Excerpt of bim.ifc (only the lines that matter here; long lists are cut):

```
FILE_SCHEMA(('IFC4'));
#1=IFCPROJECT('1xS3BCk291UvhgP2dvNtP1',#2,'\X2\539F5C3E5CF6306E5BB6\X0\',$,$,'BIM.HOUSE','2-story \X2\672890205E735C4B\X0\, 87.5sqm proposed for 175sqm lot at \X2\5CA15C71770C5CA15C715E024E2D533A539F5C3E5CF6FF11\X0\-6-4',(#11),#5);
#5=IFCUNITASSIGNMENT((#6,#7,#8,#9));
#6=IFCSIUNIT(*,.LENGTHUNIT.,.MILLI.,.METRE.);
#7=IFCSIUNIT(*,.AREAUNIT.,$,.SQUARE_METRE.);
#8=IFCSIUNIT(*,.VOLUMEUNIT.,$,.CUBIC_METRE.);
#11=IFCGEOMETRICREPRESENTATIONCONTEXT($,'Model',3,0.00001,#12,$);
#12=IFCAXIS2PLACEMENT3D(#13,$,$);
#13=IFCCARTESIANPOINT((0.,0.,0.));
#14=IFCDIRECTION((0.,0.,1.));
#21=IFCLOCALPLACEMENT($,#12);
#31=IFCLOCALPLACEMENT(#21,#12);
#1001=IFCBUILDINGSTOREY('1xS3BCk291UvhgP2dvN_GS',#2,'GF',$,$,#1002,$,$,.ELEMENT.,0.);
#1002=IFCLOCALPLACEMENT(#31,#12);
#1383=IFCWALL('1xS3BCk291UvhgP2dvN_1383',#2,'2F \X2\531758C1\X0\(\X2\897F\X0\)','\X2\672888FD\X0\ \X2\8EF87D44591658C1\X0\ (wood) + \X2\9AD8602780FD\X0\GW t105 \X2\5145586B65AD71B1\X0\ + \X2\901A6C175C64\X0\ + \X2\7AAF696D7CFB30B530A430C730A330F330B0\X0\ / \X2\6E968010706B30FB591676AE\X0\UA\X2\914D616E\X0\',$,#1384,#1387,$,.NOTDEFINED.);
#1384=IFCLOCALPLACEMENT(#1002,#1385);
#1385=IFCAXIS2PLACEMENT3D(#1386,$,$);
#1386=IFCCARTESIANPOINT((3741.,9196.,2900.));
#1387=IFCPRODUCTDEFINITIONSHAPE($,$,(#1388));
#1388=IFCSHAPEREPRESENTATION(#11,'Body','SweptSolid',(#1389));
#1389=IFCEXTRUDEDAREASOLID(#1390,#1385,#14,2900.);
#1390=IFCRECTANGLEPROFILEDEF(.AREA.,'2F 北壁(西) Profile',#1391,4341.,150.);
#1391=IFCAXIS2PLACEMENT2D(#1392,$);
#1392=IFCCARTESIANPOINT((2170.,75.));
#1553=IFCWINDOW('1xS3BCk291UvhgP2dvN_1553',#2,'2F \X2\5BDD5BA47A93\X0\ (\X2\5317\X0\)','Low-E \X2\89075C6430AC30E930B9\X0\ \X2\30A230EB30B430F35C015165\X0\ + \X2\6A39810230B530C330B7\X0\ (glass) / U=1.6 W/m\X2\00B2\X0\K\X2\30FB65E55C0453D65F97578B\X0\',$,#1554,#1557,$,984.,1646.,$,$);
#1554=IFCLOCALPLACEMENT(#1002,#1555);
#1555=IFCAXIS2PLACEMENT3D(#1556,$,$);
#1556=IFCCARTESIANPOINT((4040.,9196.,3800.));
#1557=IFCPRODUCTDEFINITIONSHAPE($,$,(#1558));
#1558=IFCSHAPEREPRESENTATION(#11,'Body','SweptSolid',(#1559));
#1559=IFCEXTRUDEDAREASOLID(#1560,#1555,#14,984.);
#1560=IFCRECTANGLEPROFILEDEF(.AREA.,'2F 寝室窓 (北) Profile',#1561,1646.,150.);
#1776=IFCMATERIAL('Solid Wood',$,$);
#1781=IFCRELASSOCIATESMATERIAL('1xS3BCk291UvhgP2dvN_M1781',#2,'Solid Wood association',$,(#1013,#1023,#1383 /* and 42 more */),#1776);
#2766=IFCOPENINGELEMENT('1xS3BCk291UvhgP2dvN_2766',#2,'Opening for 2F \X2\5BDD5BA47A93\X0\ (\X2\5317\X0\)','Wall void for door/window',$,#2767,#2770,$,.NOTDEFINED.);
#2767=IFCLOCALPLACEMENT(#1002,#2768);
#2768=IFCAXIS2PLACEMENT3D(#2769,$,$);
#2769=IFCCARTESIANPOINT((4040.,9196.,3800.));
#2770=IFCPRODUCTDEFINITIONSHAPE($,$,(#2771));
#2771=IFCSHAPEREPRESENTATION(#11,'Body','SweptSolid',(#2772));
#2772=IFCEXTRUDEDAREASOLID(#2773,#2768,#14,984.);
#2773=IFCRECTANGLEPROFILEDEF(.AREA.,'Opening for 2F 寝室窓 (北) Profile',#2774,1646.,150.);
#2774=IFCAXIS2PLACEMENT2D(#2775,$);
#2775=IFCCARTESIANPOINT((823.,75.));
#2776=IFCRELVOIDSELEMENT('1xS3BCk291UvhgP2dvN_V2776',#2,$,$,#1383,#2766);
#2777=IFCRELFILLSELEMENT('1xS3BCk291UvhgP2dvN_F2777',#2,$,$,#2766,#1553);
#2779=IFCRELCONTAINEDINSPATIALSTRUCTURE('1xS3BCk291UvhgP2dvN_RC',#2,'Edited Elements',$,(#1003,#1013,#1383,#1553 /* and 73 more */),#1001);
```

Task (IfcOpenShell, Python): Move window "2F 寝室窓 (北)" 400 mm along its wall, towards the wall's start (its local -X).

```python
import ifcopenshell
import ifcopenshell.api.geometry
import ifcopenshell.util.placement
import ifcopenshell.util.unit

model = ifcopenshell.open("bim.ifc")
unit_scale = ifcopenshell.util.unit.calculate_unit_scale(model)

window = model.by_guid("1xS3BCk291UvhgP2dvN_1553")
opening = window.FillsVoids[0].RelatingOpeningElement
wall = opening.VoidsElements[0].RelatingBuildingElement

wall_matrix = ifcopenshell.util.placement.get_local_placement(wall.ObjectPlacement)
shift = wall_matrix[:3, 0] * -0.4 / unit_scale
before = ifcopenshell.util.placement.get_local_placement(window.ObjectPlacement)[:3, 3].copy()

# The window is not placed relative to its opening, so move both.
for product in (opening, window):
    matrix = ifcopenshell.util.placement.get_local_placement(product.ObjectPlacement)
    matrix[:3, 3] += shift
    ifcopenshell.api.geometry.edit_object_placement(model, product=product, matrix=matrix, is_si=False)

after = ifcopenshell.util.placement.get_local_placement(window.ObjectPlacement)[:3, 3]
print("window moved by", (after - before).round(3) + 0.0)

model.write("bim_rev.ifc")
```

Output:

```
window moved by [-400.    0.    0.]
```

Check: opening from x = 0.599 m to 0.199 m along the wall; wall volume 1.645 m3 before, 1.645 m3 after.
